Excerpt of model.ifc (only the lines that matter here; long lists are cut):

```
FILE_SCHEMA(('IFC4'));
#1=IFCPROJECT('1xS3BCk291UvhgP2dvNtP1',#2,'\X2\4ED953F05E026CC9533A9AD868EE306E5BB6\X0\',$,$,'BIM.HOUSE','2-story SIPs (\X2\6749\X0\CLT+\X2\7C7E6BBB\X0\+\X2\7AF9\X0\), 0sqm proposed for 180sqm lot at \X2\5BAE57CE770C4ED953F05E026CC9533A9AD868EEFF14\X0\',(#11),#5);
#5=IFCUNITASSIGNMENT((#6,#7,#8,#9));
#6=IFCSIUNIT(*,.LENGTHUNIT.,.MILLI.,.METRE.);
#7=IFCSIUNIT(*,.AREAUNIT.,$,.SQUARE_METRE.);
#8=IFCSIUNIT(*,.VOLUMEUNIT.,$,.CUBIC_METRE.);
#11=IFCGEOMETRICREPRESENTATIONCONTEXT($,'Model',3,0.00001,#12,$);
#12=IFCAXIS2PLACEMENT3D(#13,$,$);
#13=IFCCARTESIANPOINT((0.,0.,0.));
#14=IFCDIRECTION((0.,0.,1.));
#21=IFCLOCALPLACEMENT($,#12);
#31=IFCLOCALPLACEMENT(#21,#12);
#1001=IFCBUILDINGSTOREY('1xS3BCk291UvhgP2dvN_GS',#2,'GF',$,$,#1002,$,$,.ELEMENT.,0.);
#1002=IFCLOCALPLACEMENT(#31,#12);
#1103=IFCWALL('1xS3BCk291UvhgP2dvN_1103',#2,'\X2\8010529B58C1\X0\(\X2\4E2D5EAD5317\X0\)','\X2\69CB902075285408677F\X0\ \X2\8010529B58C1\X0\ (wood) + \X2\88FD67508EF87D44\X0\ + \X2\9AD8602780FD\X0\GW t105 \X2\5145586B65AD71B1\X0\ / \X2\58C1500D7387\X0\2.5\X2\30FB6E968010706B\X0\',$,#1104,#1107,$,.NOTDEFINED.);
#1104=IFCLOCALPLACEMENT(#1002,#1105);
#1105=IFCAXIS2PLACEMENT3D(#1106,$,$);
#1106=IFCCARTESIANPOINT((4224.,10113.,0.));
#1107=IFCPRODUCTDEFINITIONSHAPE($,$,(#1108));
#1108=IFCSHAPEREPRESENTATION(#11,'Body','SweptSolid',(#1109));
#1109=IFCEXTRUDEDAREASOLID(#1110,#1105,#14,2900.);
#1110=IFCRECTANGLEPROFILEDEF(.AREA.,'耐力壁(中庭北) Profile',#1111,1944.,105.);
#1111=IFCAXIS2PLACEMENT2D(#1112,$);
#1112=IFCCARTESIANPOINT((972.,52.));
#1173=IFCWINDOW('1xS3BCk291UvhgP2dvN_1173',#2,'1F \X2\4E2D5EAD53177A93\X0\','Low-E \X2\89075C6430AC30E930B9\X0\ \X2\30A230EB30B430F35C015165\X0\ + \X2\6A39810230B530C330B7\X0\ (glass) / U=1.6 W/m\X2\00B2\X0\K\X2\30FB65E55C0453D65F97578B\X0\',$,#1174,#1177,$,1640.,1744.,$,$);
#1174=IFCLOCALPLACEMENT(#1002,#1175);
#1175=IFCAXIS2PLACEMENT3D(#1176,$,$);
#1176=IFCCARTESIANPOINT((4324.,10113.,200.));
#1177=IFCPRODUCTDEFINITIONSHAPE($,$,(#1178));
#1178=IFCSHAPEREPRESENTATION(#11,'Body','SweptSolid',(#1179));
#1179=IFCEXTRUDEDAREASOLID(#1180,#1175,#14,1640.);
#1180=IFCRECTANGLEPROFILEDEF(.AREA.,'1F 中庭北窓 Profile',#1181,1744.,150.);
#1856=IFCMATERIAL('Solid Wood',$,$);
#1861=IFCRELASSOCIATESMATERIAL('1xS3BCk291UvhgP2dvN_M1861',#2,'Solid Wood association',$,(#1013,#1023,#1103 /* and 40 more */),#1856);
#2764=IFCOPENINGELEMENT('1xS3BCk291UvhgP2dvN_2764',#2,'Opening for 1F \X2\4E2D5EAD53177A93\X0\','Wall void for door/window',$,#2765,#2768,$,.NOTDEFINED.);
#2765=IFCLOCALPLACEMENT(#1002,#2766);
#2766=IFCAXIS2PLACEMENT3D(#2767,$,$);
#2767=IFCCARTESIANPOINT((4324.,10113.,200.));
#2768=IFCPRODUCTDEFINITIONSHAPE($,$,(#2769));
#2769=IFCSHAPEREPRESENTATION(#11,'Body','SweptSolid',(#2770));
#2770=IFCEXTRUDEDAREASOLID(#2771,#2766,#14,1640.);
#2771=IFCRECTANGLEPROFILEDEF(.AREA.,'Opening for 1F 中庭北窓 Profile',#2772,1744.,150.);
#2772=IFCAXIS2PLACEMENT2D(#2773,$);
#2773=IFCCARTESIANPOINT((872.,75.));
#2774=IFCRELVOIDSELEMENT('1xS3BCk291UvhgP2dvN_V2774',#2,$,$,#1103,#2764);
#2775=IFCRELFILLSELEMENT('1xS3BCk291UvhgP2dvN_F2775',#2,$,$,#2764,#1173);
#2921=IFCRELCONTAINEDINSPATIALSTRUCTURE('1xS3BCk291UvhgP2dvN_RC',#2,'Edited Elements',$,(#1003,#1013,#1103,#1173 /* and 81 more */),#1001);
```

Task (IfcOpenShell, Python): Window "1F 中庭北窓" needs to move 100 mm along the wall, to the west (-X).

```python
import ifcopenshell
import ifcopenshell.api.geometry
import ifcopenshell.util.placement

model = ifcopenshell.open("model.ifc")

window = model.by_id(1173)
opening = window.FillsVoids[0].RelatingOpeningElement
wall = opening.VoidsElements[0].RelatingBuildingElement

wall_matrix = ifcopenshell.util.placement.get_local_placement(wall.ObjectPlacement)
shift = wall_matrix[:3, 0] * -100.0
before = ifcopenshell.util.placement.get_local_placement(window.ObjectPlacement)[:3, 3].copy()

# The window is not placed relative to its opening, so move both.
for product in (opening, window):
    matrix = ifcopenshell.util.placement.get_local_placement(product.ObjectPlacement)
    matrix[:3, 3] += shift
    ifcopenshell.api.geometry.edit_object_placement(model, product=product, matrix=matrix, is_si=False)

after = ifcopenshell.util.placement.get_local_placement(window.ObjectPlacement)[:3, 3]
print("window moved by", (after - before).round(3) + 0.0)

model.write("model_rev.ifc")
```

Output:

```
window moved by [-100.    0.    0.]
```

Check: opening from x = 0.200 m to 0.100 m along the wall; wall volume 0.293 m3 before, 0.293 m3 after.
